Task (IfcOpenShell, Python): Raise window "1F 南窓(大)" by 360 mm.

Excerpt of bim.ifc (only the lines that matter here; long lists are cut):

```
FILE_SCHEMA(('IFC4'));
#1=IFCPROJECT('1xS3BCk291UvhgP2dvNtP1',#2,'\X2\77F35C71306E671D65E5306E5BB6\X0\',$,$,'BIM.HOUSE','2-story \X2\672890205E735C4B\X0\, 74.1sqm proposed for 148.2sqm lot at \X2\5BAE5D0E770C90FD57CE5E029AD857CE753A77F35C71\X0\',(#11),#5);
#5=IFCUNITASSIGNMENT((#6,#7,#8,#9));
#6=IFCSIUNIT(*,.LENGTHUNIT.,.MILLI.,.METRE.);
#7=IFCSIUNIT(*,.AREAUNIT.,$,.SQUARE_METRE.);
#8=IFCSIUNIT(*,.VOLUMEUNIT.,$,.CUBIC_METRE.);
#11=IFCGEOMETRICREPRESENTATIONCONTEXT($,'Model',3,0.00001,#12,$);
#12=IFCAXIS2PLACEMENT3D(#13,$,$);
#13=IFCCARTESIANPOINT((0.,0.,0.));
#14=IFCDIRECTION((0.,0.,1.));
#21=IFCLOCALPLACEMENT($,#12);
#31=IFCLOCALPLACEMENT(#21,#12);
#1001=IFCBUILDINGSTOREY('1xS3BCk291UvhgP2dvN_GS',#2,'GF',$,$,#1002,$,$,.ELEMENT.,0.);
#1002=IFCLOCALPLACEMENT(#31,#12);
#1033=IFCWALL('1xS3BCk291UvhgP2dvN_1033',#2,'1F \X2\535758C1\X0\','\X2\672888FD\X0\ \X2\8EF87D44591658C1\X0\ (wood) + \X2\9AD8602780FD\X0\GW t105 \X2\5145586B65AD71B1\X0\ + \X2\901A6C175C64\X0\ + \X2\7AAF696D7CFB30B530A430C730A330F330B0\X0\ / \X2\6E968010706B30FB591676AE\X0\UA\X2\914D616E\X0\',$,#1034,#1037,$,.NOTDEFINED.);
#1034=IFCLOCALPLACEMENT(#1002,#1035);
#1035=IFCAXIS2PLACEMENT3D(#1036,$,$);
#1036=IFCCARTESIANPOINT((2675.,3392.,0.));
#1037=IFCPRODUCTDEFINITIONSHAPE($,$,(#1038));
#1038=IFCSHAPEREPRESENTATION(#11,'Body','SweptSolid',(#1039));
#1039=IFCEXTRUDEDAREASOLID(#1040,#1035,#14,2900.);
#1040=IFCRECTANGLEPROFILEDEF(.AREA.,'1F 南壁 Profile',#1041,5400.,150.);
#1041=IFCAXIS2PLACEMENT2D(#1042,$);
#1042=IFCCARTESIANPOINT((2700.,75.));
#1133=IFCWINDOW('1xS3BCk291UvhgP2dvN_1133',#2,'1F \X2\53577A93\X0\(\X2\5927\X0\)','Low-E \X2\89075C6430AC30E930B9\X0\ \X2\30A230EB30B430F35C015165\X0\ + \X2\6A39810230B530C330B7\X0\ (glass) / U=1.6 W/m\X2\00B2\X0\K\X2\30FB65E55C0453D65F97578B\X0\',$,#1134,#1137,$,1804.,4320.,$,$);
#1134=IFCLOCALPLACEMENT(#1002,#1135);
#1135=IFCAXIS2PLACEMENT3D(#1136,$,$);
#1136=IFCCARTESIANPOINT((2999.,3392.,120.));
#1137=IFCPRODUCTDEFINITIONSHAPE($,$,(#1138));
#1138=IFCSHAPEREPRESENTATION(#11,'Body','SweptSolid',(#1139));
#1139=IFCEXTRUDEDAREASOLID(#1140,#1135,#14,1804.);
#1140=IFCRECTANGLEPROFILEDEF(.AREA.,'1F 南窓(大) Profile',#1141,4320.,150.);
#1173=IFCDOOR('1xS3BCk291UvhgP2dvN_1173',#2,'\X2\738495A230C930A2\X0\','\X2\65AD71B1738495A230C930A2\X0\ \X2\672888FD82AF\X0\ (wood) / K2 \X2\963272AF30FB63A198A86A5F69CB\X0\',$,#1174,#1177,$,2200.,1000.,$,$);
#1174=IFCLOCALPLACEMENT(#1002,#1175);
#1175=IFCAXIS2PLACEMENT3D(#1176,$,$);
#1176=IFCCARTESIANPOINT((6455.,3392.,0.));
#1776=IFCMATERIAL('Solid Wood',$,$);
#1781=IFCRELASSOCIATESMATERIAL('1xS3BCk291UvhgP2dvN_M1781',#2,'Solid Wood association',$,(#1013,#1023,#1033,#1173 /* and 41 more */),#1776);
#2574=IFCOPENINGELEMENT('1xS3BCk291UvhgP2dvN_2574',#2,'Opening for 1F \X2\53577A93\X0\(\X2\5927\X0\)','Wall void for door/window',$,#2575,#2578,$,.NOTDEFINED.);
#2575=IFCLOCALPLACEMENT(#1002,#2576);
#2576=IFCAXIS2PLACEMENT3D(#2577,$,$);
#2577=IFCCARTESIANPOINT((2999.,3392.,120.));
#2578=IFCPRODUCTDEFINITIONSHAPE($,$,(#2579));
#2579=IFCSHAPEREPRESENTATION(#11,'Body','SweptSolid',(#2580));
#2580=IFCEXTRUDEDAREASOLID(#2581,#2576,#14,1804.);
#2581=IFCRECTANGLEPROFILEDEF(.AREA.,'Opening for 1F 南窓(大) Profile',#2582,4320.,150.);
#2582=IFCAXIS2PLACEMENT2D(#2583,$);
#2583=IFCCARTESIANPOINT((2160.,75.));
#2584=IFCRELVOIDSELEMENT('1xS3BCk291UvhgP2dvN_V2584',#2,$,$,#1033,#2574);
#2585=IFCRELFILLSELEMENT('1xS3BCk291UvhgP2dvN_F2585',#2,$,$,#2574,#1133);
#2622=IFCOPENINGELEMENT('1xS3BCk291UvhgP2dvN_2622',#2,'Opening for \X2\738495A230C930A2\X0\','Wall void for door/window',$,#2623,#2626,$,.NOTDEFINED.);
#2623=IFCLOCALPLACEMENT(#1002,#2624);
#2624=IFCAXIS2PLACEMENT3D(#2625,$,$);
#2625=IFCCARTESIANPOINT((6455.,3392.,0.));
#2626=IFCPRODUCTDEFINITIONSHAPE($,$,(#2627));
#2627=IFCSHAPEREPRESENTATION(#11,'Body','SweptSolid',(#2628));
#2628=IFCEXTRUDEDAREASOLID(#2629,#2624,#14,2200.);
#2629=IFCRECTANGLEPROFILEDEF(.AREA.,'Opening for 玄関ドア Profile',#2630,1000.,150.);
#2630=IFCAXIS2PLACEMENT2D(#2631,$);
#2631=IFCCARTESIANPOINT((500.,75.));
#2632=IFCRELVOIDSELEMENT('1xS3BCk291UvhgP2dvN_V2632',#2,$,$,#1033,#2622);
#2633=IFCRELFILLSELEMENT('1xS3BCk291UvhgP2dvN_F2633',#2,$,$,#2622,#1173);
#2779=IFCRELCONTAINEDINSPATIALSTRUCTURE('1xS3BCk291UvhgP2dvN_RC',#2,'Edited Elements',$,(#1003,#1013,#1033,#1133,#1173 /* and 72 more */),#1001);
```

```python
import numpy as np
import ifcopenshell
import ifcopenshell.api.geometry
import ifcopenshell.util.placement
import ifcopenshell.util.unit

model = ifcopenshell.open("bim.ifc")
unit_scale = ifcopenshell.util.unit.calculate_unit_scale(model)

window = model.by_guid("1xS3BCk291UvhgP2dvN_1133")
opening = window.FillsVoids[0].RelatingOpeningElement
dz = 0.36 / unit_scale

shift = np.array([0.0, 0.0, dz])
# The window is not placed relative to its opening, so move both.
for product in (opening, window):
    matrix = ifcopenshell.util.placement.get_local_placement(product.ObjectPlacement)
    matrix[:3, 3] += shift
    ifcopenshell.api.geometry.edit_object_placement(model, product=product, matrix=matrix, is_si=False)

print(f"moved by {dz * unit_scale:+.3f} m")

model.write("bim_rev.ifc")
```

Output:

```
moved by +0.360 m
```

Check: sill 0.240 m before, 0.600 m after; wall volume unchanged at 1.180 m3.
